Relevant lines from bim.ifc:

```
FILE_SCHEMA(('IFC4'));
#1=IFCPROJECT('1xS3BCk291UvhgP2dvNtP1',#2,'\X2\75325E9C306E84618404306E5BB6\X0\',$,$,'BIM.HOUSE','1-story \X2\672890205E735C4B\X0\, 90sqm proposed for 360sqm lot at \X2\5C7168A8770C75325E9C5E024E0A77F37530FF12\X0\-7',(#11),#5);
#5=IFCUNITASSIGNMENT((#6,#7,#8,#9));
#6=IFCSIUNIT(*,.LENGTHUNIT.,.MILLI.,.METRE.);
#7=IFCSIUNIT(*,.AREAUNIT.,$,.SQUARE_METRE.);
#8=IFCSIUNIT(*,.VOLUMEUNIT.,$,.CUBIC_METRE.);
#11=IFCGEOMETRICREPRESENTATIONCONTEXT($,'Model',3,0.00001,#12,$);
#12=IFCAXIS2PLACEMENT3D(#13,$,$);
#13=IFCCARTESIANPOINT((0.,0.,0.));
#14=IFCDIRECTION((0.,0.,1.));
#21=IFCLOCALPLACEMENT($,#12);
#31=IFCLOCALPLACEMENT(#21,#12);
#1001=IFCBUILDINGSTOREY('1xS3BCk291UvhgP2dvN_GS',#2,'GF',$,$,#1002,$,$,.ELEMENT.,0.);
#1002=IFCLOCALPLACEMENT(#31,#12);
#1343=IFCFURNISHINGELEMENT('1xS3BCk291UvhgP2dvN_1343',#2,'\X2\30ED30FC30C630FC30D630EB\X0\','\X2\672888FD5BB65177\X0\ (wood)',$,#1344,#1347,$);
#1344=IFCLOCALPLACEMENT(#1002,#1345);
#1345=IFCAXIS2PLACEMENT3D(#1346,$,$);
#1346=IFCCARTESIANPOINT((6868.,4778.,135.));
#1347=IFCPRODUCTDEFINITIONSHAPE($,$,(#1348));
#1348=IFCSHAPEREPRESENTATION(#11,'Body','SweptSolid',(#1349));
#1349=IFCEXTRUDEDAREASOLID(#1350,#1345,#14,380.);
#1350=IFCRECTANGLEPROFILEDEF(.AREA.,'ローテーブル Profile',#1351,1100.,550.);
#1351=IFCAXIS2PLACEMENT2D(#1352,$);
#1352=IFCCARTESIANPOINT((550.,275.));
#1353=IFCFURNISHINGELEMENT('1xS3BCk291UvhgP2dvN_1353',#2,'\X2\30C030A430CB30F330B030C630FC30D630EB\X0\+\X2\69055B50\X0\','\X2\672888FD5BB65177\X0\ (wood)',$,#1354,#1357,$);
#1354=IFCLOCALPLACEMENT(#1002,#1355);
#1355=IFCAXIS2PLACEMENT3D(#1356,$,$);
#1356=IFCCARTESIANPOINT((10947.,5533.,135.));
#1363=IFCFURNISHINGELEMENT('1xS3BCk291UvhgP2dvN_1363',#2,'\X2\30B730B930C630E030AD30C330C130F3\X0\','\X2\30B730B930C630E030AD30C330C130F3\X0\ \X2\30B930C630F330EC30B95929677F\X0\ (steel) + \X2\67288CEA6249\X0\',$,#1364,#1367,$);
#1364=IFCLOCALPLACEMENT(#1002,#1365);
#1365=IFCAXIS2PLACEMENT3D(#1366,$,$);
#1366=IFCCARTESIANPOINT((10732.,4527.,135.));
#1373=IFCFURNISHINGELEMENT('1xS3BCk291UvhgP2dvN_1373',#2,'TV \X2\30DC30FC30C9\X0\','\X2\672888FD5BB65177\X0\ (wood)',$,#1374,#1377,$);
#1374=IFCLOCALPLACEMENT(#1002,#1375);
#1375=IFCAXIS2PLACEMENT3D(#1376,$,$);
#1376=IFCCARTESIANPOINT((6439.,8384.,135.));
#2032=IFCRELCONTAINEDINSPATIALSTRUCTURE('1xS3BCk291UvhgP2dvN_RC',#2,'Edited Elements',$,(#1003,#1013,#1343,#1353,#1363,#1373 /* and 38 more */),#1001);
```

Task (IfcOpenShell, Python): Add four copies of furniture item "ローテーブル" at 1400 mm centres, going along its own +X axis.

```python
import ifcopenshell
import ifcopenshell.api.geometry
import ifcopenshell.api.root
import ifcopenshell.util.element
import ifcopenshell.util.placement
import ifcopenshell.util.unit

model = ifcopenshell.open("bim.ifc")
unit_scale = ifcopenshell.util.unit.calculate_unit_scale(model)


def reuse_history(source, copy):
    """copy_class also copies each property set's owner history, people and application; keep the originals."""
    for rel in copy.IsDefinedBy:
        if rel.is_a("IfcRelDefinesByProperties") and (history := rel.RelatingPropertyDefinition.OwnerHistory):
            rel.RelatingPropertyDefinition.OwnerHistory = source.OwnerHistory
            ifcopenshell.util.element.remove_deep2(model, history)


source = model.by_guid("1xS3BCk291UvhgP2dvN_1343")
base = ifcopenshell.util.placement.get_local_placement(source.ObjectPlacement)
step = base[:3, 0] * 1.4 / unit_scale

for i in range(1, 5):
    copy = ifcopenshell.api.root.copy_class(model, product=source)
    copy.Representation = ifcopenshell.util.element.copy_deep(
        model, source.Representation, exclude=["IfcGeometricRepresentationContext", "IfcRepresentationMap"]
    )
    reuse_history(source, copy)
    matrix = base.copy()
    matrix[:3, 3] += i * step
    print("added at", matrix[:3, 3].round(3) + 0.0)
    ifcopenshell.api.geometry.edit_object_placement(model, product=copy, matrix=matrix, is_si=False)

model.write("bim-out.ifc")
```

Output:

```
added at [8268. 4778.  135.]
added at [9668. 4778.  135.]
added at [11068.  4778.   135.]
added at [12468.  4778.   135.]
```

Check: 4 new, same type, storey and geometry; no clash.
